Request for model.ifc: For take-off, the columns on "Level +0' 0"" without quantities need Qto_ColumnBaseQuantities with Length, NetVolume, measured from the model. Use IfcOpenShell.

First a look at what the model holds.

```python
import ifcopenshell
import ifcopenshell.util.element
import ifcopenshell.util.unit

model = ifcopenshell.open("model.ifc")
print(model.schema)
for unit_type in ("LENGTHUNIT", "AREAUNIT", "VOLUMEUNIT"):
    print(unit_type, ifcopenshell.util.unit.calculate_unit_scale(model, unit_type))
storey = next(s for s in model.by_type("IfcBuildingStorey") if s.Name == 'Level +0\' 0"')
columns = [e for e in ifcopenshell.util.element.get_decomposition(storey) if e.is_a("IfcColumn")]
for e in sorted(columns, key=lambda e: e.id()):
    print(e.id(), e.is_a(), e.Name, list(ifcopenshell.util.element.get_psets(e, qtos_only=True)), sep=" | ")
```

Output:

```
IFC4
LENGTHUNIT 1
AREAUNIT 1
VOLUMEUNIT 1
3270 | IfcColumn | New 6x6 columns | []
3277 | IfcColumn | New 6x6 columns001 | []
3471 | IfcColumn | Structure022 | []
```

```python
import ifcopenshell
import ifcopenshell.api.pset
import ifcopenshell.geom
import ifcopenshell.util.element
import ifcopenshell.util.shape
import ifcopenshell.util.unit

model = ifcopenshell.open("model.ifc")
unit_scale = ifcopenshell.util.unit.calculate_unit_scale(model)
volume_scale = ifcopenshell.util.unit.calculate_unit_scale(model, "VOLUMEUNIT")
settings = ifcopenshell.geom.settings()

storey = next(s for s in model.by_type("IfcBuildingStorey") if s.Name == 'Level +0\' 0"')
columns = [e for e in ifcopenshell.util.element.get_decomposition(storey) if e.is_a("IfcColumn")]

for e in sorted(columns, key=lambda e: e.id()):
    if ifcopenshell.util.element.get_psets(e, qtos_only=True, should_inherit=False):
        continue
    # Geometry comes back in metres, in the element's own axes.
    shape = ifcopenshell.geom.create_shape(settings, e)
    values = {
        "Length": ifcopenshell.util.shape.get_z(shape.geometry) / unit_scale,
        "NetVolume": ifcopenshell.util.shape.get_volume(shape.geometry) / volume_scale,
    }
    qto = ifcopenshell.api.pset.add_qto(model, product=e, name="Qto_ColumnBaseQuantities")
    ifcopenshell.api.pset.edit_qto(model, qto=qto, properties=values)
    print(e.id(), {k: round(v, 3) for k, v in values.items()})

model.write("model_rev.ifc")
```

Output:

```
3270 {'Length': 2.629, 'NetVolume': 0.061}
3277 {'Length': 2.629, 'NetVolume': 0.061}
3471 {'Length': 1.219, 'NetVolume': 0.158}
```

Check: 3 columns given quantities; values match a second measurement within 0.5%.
